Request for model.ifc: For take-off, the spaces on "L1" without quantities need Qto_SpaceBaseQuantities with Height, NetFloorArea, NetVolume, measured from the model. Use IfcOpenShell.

First a look at what the model holds.

```python
import ifcopenshell
import ifcopenshell.util.element
import ifcopenshell.util.unit

model = ifcopenshell.open("model.ifc")
print(model.schema)
for unit_type in ("LENGTHUNIT", "AREAUNIT", "VOLUMEUNIT"):
    print(unit_type, ifcopenshell.util.unit.calculate_unit_scale(model, unit_type))
storey = next(s for s in model.by_type("IfcBuildingStorey") if s.Name == "L1")
spaces = [e for e in ifcopenshell.util.element.get_decomposition(storey) if e.is_a("IfcSpace")]
for e in sorted(spaces, key=lambda e: e.id()):
    print(e.id(), e.is_a(), e.Name, list(ifcopenshell.util.element.get_psets(e, qtos_only=True)), sep=" | ")
```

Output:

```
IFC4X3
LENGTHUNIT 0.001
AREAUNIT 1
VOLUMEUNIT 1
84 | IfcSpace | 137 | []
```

```python
import ifcopenshell
import ifcopenshell.api.pset
import ifcopenshell.geom
import ifcopenshell.util.element
import ifcopenshell.util.shape
import ifcopenshell.util.unit

model = ifcopenshell.open("model.ifc")
unit_scale = ifcopenshell.util.unit.calculate_unit_scale(model)
area_scale = ifcopenshell.util.unit.calculate_unit_scale(model, "AREAUNIT")
volume_scale = ifcopenshell.util.unit.calculate_unit_scale(model, "VOLUMEUNIT")
settings = ifcopenshell.geom.settings()

storey = next(s for s in model.by_type("IfcBuildingStorey") if s.Name == "L1")
spaces = [e for e in ifcopenshell.util.element.get_decomposition(storey) if e.is_a("IfcSpace")]

for e in sorted(spaces, key=lambda e: e.id()):
    if ifcopenshell.util.element.get_psets(e, qtos_only=True, should_inherit=False):
        continue
    # Geometry comes back in metres, in the element's own axes.
    shape = ifcopenshell.geom.create_shape(settings, e)
    values = {
        "Height": ifcopenshell.util.shape.get_z(shape.geometry) / unit_scale,
        "NetFloorArea": ifcopenshell.util.shape.get_footprint_area(shape.geometry) / area_scale,
        "NetVolume": ifcopenshell.util.shape.get_volume(shape.geometry) / volume_scale,
    }
    qto = ifcopenshell.api.pset.add_qto(model, product=e, name="Qto_SpaceBaseQuantities")
    ifcopenshell.api.pset.edit_qto(model, qto=qto, properties=values)
    print(e.id(), {k: round(v, 3) for k, v in values.items()})

model.write("model-out.ifc")
```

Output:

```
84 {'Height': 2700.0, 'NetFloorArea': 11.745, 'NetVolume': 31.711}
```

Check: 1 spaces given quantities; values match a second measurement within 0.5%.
